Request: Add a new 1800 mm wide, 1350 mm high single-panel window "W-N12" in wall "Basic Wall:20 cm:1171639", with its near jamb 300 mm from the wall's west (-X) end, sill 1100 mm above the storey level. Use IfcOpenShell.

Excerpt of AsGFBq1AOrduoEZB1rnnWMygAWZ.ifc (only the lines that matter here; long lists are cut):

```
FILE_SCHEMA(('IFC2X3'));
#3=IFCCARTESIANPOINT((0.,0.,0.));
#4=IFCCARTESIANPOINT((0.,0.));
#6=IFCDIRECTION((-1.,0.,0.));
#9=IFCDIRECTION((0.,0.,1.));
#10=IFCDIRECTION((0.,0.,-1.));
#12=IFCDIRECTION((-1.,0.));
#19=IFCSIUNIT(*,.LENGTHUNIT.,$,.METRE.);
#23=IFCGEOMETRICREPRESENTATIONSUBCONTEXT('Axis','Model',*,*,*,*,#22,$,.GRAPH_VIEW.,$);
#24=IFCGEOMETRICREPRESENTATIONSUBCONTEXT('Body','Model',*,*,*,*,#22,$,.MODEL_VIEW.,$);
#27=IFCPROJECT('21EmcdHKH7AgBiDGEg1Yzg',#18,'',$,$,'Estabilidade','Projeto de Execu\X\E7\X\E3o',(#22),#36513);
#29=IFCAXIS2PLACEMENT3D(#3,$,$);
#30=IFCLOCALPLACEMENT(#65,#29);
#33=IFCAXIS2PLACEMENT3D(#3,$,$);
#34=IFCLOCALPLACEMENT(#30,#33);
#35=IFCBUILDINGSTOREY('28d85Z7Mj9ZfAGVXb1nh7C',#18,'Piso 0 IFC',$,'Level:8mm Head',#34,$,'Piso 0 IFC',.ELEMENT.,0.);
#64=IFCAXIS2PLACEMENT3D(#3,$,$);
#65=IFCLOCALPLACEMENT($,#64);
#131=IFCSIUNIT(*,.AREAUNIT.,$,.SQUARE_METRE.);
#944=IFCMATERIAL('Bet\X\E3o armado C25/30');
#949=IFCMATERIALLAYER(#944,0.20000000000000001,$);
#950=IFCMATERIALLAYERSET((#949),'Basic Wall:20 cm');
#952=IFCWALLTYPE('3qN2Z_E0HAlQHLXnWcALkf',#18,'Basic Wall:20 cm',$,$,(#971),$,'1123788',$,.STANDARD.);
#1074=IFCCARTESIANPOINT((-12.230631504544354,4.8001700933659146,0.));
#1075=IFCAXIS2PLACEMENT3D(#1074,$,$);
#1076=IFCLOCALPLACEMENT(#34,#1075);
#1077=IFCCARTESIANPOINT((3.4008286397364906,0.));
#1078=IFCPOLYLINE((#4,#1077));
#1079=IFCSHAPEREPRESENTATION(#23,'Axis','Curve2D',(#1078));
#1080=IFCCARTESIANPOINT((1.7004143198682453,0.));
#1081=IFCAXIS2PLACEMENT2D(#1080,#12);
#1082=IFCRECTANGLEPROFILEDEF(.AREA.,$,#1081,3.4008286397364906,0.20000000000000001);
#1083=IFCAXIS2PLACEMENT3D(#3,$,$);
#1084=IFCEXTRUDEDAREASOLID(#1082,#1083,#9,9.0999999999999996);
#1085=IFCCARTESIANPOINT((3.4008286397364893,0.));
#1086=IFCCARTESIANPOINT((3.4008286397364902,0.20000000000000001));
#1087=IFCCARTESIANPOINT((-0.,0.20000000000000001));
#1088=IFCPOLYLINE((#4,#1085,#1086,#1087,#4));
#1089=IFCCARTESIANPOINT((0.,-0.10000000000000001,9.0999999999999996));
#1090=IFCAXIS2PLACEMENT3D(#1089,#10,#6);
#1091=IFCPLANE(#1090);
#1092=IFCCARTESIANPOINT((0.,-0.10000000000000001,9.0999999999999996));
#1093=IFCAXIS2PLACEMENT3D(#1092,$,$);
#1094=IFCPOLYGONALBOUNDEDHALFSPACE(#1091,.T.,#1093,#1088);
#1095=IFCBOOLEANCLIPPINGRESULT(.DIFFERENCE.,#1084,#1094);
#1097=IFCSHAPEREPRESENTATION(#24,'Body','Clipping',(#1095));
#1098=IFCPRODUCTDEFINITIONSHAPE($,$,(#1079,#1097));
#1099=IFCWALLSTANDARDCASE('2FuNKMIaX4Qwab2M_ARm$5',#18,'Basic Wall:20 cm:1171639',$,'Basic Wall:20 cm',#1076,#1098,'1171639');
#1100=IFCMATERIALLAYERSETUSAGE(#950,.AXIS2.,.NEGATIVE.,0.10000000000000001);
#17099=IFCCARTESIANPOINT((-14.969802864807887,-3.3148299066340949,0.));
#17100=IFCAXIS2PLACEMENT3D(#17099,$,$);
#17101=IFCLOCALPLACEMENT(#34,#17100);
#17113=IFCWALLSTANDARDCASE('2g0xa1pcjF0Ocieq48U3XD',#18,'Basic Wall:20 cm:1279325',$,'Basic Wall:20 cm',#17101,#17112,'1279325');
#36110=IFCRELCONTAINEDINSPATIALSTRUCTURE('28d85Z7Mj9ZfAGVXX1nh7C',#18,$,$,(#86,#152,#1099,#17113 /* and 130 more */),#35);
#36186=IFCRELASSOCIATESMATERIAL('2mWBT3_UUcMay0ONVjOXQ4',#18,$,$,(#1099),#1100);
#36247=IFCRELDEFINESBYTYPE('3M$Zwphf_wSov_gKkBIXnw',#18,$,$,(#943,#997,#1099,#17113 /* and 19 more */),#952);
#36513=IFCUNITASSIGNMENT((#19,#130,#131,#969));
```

```python
import numpy as np
import ifcopenshell
import ifcopenshell.api.feature
import ifcopenshell.api.geometry
import ifcopenshell.api.root
import ifcopenshell.api.spatial
import ifcopenshell.api.type
import ifcopenshell.geom
import ifcopenshell.util.element
import ifcopenshell.util.placement
import ifcopenshell.util.representation
import ifcopenshell.util.shape
import ifcopenshell.util.unit

model = ifcopenshell.open("AsGFBq1AOrduoEZB1rnnWMygAWZ.ifc")
unit_scale = ifcopenshell.util.unit.calculate_unit_scale(model)
settings = ifcopenshell.geom.settings()


def volume(element):
    """Net volume in cubic metres, openings subtracted."""
    shape = ifcopenshell.geom.create_shape(settings, element)
    return ifcopenshell.util.shape.get_volume(shape.geometry)


wall = model.by_id(1099)
storey = ifcopenshell.util.element.get_container(wall, ifc_class="IfcBuildingStorey")
context = ifcopenshell.util.representation.get_context(model, "Model", "Body", "MODEL_VIEW")
before = volume(wall)

width, height, from_end, sill = 1.8, 1.35, 0.3, 1.1  # metres

# The wall runs along its own X axis, and the end named is its -X end.
wall_shape = ifcopenshell.geom.create_shape(settings, wall)
x, y, z = ifcopenshell.util.shape.get_vertices(wall_shape.geometry).T
start = x.min() + from_end
face, thickness = float(y.min()), float(y.max() - y.min())
wall_matrix = ifcopenshell.util.placement.get_local_placement(wall.ObjectPlacement)
level = ifcopenshell.util.placement.get_local_placement(storey.ObjectPlacement)[2, 3]


def in_wall(x, y):
    """Placement at x, y metres in the wall's axes, at sill height."""
    matrix = wall_matrix.copy()
    matrix[:, 3] = wall_matrix @ np.array([x / unit_scale, y / unit_scale, 0.0, 1.0])
    matrix[2, 3] = level + sill / unit_scale
    return matrix


# Opening: a box that overshoots both wall faces by 50 mm.
opening = ifcopenshell.api.root.create_entity(model, ifc_class="IfcOpeningElement")
box = ifcopenshell.api.geometry.add_wall_representation(
    model, context=context, length=width, height=height, thickness=thickness + 0.1
)
ifcopenshell.api.geometry.assign_representation(model, product=opening, representation=box)
ifcopenshell.api.geometry.edit_object_placement(model, product=opening, matrix=in_wall(start, face - 0.05), is_si=False)
ifcopenshell.api.feature.add_feature(model, feature=opening, element=wall)

window = ifcopenshell.api.root.create_entity(model, ifc_class="IfcWindow", name="W-N12")
window.OverallWidth, window.OverallHeight = width / unit_scale, height / unit_scale
body = ifcopenshell.api.geometry.add_window_representation(
    model,
    context=context,
    overall_width=window.OverallWidth,
    overall_height=window.OverallHeight,
    partition_type="SINGLE_PANEL",
)
ifcopenshell.api.geometry.assign_representation(model, product=window, representation=body)
ifcopenshell.api.spatial.assign_container(model, products=[window], relating_structure=storey)
fills = ifcopenshell.api.feature.add_filling(model, opening=opening, element=window)
fills.OwnerHistory = window.OwnerHistory  # required in IFC2X3

# IFC2X3 keeps the operation on the window style.
style = ifcopenshell.api.root.create_entity(model, ifc_class="IfcWindowStyle", name="W-N12")
style.OperationType, style.ConstructionType = "SINGLE_PANEL", "NOTDEFINED"
style.ParameterTakesPrecedence = style.Sizeable = False
ifcopenshell.api.type.assign_type(model, related_objects=[window], relating_type=style)

# Centre the window in the wall's thickness.
ifcopenshell.api.geometry.edit_object_placement(model, product=window, matrix=in_wall(start, face), is_si=False)
window_shape = ifcopenshell.geom.create_shape(settings, window)
depth = ifcopenshell.util.shape.get_vertices(window_shape.geometry)[:, 1]
offset = face + thickness / 2 - (depth.min() + depth.max()) / 2
ifcopenshell.api.geometry.edit_object_placement(model, product=window, matrix=in_wall(start, offset), is_si=False)

after = volume(wall)

print(f"wall volume {before:.3f} -> {after:.3f} m3")

model.write("AsGFBq1AOrduoEZB1rnnWMygAWZ_updated.ifc")
```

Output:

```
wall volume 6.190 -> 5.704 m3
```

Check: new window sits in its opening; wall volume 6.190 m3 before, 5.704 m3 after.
